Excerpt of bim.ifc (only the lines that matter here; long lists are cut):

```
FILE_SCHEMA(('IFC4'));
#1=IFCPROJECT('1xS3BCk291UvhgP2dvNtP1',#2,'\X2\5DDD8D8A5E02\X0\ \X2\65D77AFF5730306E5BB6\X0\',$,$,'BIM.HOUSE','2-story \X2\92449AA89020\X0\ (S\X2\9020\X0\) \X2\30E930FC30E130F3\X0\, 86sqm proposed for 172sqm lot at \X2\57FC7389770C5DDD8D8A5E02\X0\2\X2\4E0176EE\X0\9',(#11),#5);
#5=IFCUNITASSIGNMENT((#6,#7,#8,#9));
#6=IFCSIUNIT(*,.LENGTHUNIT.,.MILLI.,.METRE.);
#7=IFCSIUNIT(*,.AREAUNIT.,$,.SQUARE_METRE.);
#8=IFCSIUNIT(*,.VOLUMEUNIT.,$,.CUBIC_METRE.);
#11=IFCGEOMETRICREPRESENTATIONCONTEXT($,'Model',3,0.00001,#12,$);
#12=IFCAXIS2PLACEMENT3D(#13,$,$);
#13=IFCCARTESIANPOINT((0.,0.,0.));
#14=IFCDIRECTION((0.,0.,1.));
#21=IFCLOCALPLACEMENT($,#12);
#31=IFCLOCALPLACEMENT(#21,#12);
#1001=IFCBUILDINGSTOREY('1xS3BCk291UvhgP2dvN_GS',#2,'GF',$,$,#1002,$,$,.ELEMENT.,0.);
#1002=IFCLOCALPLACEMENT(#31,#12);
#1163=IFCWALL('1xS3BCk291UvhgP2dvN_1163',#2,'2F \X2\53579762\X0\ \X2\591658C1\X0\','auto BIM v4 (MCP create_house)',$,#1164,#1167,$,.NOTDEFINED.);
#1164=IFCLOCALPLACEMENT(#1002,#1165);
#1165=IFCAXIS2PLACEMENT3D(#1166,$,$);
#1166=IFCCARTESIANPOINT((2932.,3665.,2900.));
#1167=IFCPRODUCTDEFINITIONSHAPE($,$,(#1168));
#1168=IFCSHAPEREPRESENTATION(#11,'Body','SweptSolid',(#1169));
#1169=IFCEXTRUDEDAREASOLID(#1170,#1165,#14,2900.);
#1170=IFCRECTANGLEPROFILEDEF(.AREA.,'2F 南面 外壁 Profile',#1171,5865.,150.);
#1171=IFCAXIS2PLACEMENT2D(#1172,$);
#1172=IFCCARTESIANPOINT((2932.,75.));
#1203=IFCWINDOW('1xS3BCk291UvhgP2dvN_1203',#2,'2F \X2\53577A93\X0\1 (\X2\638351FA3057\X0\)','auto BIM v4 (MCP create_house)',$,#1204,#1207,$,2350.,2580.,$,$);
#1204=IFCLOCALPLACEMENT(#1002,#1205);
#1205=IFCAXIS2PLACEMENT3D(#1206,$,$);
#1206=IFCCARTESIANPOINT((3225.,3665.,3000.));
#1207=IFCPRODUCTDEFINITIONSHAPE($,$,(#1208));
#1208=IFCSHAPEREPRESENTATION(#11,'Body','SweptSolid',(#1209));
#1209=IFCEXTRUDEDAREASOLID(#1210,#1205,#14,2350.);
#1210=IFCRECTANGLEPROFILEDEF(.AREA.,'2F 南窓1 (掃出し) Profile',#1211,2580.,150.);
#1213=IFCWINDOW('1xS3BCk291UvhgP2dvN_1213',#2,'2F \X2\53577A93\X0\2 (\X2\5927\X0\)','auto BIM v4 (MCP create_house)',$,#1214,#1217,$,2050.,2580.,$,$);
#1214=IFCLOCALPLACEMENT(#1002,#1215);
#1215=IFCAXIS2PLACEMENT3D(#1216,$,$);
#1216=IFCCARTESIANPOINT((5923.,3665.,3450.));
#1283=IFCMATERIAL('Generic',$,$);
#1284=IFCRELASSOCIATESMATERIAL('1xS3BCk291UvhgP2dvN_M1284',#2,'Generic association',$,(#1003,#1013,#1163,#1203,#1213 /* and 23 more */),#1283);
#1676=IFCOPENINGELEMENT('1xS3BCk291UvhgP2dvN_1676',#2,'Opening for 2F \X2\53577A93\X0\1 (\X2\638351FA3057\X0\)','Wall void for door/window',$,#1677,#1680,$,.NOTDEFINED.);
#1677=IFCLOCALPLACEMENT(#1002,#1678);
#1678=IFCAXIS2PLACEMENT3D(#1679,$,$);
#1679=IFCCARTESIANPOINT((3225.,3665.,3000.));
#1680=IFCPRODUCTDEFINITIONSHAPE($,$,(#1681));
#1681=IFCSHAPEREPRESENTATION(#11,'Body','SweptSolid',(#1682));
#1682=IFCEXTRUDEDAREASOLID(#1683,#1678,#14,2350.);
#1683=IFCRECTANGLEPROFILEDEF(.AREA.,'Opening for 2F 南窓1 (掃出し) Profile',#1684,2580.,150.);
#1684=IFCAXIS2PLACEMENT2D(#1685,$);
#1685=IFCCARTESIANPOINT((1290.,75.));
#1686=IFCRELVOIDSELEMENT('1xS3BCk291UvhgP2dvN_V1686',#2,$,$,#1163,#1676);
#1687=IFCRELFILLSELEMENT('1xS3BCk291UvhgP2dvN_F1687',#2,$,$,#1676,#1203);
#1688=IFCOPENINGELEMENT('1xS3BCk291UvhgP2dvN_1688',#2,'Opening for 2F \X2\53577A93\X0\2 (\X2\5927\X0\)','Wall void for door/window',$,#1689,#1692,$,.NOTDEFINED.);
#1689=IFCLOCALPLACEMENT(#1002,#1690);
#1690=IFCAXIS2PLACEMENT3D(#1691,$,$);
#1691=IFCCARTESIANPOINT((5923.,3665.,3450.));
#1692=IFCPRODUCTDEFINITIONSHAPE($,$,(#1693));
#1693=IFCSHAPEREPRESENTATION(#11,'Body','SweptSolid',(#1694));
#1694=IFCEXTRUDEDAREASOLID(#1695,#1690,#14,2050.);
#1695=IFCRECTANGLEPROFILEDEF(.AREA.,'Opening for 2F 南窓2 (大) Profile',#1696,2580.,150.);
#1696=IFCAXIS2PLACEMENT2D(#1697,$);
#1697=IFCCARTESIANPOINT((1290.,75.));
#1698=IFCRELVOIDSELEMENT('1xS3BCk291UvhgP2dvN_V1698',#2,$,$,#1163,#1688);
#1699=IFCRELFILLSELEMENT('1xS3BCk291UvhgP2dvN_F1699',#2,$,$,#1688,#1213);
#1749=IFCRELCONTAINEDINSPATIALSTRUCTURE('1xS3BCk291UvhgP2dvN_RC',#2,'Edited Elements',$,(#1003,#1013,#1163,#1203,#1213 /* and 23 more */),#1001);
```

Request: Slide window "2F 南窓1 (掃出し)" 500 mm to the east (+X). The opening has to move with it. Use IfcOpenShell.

```python
import ifcopenshell
import ifcopenshell.api.geometry
import ifcopenshell.util.placement

model = ifcopenshell.open("bim.ifc")

window = model.by_id(1203)
opening = window.FillsVoids[0].RelatingOpeningElement
wall = opening.VoidsElements[0].RelatingBuildingElement

wall_matrix = ifcopenshell.util.placement.get_local_placement(wall.ObjectPlacement)
shift = wall_matrix[:3, 0] * 500.0
before = ifcopenshell.util.placement.get_local_placement(window.ObjectPlacement)[:3, 3].copy()

# The window is not placed relative to its opening, so move both.
for product in (opening, window):
    matrix = ifcopenshell.util.placement.get_local_placement(product.ObjectPlacement)
    matrix[:3, 3] += shift
    ifcopenshell.api.geometry.edit_object_placement(model, product=product, matrix=matrix, is_si=False)

after = ifcopenshell.util.placement.get_local_placement(window.ObjectPlacement)[:3, 3]
print("window moved by", (after - before).round(3) + 0.0)

model.write("bim_v2.ifc")
```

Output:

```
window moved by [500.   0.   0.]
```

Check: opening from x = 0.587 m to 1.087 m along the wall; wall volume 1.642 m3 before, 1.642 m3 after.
